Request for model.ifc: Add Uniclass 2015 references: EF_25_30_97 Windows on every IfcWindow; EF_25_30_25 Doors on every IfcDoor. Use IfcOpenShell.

First a look at what the model holds.

```python
import ifcopenshell

model = ifcopenshell.open("model.ifc")
print(model.schema)
print("classifications:", [c.Name for c in model.by_type("IfcClassification")])
for ifc_class in ("IfcDoor", "IfcRoof", "IfcStair", "IfcWall", "IfcWindow"):
    print(ifc_class, len(model.by_type(ifc_class)))
```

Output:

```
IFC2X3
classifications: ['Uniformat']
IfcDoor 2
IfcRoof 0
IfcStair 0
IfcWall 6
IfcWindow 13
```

```python
import ifcopenshell
import ifcopenshell.api.classification

model = ifcopenshell.open("model.ifc")

# IFC2X3 requires Source and Edition and has no link from the project to the system.
system = model.create_entity("IfcClassification", Source="NBS", Edition="2015", Name="Uniclass 2015")

codes = {
    "IfcWindow": ("EF_25_30_97", "Windows"),
    "IfcDoor": ("EF_25_30_25", "Doors"),
}
for ifc_class, (code, name) in codes.items():
    products = model.by_type(ifc_class)
    ifcopenshell.api.classification.add_reference(
        model, products=products, classification=system, identification=code, name=name
    )
    print(code, len(products))

model.write("model_updated.ifc")
```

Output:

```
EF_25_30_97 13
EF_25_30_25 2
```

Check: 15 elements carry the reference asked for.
